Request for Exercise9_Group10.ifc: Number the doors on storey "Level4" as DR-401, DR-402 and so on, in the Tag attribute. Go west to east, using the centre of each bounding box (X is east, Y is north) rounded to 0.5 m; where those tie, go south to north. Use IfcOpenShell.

First a look at what the model holds.

```python
import ifcopenshell
import ifcopenshell.util.element
import ifcopenshell.util.placement

model = ifcopenshell.open("Exercise9_Group10.ifc")
print(model.schema)
storey = next(s for s in model.by_type("IfcBuildingStorey") if s.Name == "Level4")
doors = [e for e in ifcopenshell.util.element.get_decomposition(storey) if e.is_a("IfcDoor")]
for e in sorted(doors, key=lambda e: e.id()):
    origin = ifcopenshell.util.placement.get_local_placement(e.ObjectPlacement)[:3, 3]
    print(e.id(), e.Tag, e.Name, origin.round(2) + 0.0, sep=" | ")
```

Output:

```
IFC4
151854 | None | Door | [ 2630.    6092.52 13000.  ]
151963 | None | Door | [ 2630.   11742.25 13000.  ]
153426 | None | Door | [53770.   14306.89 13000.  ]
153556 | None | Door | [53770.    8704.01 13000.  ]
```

```python
import ifcopenshell
import ifcopenshell.geom
import ifcopenshell.util.element
import ifcopenshell.util.shape

model = ifcopenshell.open("Exercise9_Group10.ifc")
settings = ifcopenshell.geom.settings()
settings.set("use-world-coords", True)


def centre(element):
    shape = ifcopenshell.geom.create_shape(settings, element)
    return ifcopenshell.util.shape.get_bbox_centroid(shape.geometry)


storey = next(s for s in model.by_type("IfcBuildingStorey") if s.Name == "Level4")
doors = [e for e in ifcopenshell.util.element.get_decomposition(storey) if e.is_a("IfcDoor")]

# Insertion points can sit at a corner or the storey origin, so sort by the geometry (in metres).
centres = {e: centre(e) for e in doors}
doors.sort(key=lambda e: (round(centres[e][0] / 0.5), centres[e][1]))

for i, e in enumerate(doors, start=1):
    number = f"DR-4{i:02d}"
    e.Tag = number
    print(e.id(), number)

model.write("Exercise9_Group10-out.ifc")
```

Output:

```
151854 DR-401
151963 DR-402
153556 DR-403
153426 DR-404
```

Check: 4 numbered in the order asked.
